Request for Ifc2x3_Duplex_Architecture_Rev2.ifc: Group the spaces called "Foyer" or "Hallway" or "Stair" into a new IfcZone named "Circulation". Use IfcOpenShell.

First a look at what the model holds.

```python
import ifcopenshell

model = ifcopenshell.open("Ifc2x3_Duplex_Architecture_Rev2.ifc")
print(model.schema)
seen = {}
for space in model.by_type("IfcSpace"):
    seen[space.LongName] = seen.get(space.LongName, 0) + 1
for name, count in sorted(seen.items(), key=str):
    print(count, "x", name)
print("zones:", [z.Name for z in model.by_type("IfcZone")][:20])
```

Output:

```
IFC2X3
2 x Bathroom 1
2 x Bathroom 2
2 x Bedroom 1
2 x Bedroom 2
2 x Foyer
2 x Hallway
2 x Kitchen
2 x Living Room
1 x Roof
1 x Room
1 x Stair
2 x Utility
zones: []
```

```python
import ifcopenshell
import ifcopenshell.api.group
import ifcopenshell.api.root

model = ifcopenshell.open("Ifc2x3_Duplex_Architecture_Rev2.ifc")

names = {"Foyer", "Hallway", "Stair"}
spaces = [s for s in model.by_type("IfcSpace") if s.LongName in names]

zone = ifcopenshell.api.root.create_entity(model, ifc_class="IfcZone", name="Circulation")
ifcopenshell.api.group.assign_group(model, products=spaces, group=zone)
print(len(spaces), "spaces in", zone.Name)

model.write("Ifc2x3_Duplex_Architecture_Rev2-out.ifc")
```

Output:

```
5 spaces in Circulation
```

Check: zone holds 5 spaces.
